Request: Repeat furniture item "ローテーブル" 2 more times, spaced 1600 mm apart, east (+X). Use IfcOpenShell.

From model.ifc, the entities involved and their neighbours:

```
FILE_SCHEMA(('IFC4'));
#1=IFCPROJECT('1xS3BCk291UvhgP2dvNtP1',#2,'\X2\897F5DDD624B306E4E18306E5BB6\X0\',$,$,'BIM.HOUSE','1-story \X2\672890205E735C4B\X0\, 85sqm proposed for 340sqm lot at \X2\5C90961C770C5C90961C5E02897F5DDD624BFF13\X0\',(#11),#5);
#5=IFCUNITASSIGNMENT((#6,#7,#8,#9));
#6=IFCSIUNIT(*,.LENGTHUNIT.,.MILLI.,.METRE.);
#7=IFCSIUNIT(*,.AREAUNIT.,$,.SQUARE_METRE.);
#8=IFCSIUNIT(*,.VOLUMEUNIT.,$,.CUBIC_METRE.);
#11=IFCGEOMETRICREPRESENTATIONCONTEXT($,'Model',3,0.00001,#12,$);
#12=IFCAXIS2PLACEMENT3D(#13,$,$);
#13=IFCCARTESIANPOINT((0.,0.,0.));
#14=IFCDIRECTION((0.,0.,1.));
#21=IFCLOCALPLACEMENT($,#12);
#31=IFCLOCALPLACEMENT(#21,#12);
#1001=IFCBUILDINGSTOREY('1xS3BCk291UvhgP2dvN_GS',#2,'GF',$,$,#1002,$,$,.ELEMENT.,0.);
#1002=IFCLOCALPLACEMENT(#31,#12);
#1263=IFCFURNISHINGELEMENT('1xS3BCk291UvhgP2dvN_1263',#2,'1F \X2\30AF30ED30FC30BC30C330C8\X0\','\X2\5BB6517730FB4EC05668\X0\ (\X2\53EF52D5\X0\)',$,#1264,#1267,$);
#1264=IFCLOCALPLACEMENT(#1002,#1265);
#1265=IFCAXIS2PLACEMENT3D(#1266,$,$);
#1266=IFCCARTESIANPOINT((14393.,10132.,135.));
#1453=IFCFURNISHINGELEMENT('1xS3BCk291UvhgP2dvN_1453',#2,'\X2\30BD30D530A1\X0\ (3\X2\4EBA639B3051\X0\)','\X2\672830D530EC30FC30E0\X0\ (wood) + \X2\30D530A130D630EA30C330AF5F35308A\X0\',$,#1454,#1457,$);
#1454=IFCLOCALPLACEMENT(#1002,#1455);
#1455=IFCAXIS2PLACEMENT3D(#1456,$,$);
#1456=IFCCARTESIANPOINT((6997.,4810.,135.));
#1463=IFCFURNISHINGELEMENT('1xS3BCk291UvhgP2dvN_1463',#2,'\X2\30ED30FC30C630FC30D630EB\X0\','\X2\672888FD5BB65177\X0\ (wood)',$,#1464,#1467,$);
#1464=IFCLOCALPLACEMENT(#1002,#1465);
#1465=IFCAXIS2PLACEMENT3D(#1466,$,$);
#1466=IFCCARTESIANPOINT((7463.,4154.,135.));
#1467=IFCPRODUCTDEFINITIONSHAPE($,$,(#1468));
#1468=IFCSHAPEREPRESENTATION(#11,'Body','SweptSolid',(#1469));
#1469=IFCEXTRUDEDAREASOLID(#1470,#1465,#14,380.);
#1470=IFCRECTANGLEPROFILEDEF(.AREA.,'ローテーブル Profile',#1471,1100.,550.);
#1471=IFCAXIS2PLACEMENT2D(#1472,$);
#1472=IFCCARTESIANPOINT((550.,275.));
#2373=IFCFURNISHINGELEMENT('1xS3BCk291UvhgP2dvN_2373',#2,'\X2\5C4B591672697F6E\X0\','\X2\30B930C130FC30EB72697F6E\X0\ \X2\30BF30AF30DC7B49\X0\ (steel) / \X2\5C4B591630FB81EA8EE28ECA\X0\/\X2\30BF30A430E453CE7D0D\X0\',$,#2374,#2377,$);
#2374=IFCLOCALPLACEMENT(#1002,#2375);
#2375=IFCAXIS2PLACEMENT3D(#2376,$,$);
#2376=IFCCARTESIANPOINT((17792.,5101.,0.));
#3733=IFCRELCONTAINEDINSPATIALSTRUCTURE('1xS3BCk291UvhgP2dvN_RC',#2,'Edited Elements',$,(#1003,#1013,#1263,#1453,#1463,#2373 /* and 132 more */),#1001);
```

```python
import numpy as np
import ifcopenshell
import ifcopenshell.api.geometry
import ifcopenshell.api.root
import ifcopenshell.util.element
import ifcopenshell.util.placement
import ifcopenshell.util.unit

model = ifcopenshell.open("model.ifc")
unit_scale = ifcopenshell.util.unit.calculate_unit_scale(model)


def reuse_history(source, copy):
    """copy_class also copies each property set's owner history, people and application; keep the originals."""
    for rel in copy.IsDefinedBy:
        if rel.is_a("IfcRelDefinesByProperties") and (history := rel.RelatingPropertyDefinition.OwnerHistory):
            rel.RelatingPropertyDefinition.OwnerHistory = source.OwnerHistory
            ifcopenshell.util.element.remove_deep2(model, history)


source = model.by_guid("1xS3BCk291UvhgP2dvN_1463")
base = ifcopenshell.util.placement.get_local_placement(source.ObjectPlacement)
step = np.array([1.0, 0.0, 0.0]) * 1.6 / unit_scale

for i in range(1, 3):
    copy = ifcopenshell.api.root.copy_class(model, product=source)
    copy.Representation = ifcopenshell.util.element.copy_deep(
        model, source.Representation, exclude=["IfcGeometricRepresentationContext", "IfcRepresentationMap"]
    )
    reuse_history(source, copy)
    matrix = base.copy()
    matrix[:3, 3] += i * step
    print("added at", matrix[:3, 3].round(3) + 0.0)
    ifcopenshell.api.geometry.edit_object_placement(model, product=copy, matrix=matrix, is_si=False)

model.write("model_updated.ifc")
```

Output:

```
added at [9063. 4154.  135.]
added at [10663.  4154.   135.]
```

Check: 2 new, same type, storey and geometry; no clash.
